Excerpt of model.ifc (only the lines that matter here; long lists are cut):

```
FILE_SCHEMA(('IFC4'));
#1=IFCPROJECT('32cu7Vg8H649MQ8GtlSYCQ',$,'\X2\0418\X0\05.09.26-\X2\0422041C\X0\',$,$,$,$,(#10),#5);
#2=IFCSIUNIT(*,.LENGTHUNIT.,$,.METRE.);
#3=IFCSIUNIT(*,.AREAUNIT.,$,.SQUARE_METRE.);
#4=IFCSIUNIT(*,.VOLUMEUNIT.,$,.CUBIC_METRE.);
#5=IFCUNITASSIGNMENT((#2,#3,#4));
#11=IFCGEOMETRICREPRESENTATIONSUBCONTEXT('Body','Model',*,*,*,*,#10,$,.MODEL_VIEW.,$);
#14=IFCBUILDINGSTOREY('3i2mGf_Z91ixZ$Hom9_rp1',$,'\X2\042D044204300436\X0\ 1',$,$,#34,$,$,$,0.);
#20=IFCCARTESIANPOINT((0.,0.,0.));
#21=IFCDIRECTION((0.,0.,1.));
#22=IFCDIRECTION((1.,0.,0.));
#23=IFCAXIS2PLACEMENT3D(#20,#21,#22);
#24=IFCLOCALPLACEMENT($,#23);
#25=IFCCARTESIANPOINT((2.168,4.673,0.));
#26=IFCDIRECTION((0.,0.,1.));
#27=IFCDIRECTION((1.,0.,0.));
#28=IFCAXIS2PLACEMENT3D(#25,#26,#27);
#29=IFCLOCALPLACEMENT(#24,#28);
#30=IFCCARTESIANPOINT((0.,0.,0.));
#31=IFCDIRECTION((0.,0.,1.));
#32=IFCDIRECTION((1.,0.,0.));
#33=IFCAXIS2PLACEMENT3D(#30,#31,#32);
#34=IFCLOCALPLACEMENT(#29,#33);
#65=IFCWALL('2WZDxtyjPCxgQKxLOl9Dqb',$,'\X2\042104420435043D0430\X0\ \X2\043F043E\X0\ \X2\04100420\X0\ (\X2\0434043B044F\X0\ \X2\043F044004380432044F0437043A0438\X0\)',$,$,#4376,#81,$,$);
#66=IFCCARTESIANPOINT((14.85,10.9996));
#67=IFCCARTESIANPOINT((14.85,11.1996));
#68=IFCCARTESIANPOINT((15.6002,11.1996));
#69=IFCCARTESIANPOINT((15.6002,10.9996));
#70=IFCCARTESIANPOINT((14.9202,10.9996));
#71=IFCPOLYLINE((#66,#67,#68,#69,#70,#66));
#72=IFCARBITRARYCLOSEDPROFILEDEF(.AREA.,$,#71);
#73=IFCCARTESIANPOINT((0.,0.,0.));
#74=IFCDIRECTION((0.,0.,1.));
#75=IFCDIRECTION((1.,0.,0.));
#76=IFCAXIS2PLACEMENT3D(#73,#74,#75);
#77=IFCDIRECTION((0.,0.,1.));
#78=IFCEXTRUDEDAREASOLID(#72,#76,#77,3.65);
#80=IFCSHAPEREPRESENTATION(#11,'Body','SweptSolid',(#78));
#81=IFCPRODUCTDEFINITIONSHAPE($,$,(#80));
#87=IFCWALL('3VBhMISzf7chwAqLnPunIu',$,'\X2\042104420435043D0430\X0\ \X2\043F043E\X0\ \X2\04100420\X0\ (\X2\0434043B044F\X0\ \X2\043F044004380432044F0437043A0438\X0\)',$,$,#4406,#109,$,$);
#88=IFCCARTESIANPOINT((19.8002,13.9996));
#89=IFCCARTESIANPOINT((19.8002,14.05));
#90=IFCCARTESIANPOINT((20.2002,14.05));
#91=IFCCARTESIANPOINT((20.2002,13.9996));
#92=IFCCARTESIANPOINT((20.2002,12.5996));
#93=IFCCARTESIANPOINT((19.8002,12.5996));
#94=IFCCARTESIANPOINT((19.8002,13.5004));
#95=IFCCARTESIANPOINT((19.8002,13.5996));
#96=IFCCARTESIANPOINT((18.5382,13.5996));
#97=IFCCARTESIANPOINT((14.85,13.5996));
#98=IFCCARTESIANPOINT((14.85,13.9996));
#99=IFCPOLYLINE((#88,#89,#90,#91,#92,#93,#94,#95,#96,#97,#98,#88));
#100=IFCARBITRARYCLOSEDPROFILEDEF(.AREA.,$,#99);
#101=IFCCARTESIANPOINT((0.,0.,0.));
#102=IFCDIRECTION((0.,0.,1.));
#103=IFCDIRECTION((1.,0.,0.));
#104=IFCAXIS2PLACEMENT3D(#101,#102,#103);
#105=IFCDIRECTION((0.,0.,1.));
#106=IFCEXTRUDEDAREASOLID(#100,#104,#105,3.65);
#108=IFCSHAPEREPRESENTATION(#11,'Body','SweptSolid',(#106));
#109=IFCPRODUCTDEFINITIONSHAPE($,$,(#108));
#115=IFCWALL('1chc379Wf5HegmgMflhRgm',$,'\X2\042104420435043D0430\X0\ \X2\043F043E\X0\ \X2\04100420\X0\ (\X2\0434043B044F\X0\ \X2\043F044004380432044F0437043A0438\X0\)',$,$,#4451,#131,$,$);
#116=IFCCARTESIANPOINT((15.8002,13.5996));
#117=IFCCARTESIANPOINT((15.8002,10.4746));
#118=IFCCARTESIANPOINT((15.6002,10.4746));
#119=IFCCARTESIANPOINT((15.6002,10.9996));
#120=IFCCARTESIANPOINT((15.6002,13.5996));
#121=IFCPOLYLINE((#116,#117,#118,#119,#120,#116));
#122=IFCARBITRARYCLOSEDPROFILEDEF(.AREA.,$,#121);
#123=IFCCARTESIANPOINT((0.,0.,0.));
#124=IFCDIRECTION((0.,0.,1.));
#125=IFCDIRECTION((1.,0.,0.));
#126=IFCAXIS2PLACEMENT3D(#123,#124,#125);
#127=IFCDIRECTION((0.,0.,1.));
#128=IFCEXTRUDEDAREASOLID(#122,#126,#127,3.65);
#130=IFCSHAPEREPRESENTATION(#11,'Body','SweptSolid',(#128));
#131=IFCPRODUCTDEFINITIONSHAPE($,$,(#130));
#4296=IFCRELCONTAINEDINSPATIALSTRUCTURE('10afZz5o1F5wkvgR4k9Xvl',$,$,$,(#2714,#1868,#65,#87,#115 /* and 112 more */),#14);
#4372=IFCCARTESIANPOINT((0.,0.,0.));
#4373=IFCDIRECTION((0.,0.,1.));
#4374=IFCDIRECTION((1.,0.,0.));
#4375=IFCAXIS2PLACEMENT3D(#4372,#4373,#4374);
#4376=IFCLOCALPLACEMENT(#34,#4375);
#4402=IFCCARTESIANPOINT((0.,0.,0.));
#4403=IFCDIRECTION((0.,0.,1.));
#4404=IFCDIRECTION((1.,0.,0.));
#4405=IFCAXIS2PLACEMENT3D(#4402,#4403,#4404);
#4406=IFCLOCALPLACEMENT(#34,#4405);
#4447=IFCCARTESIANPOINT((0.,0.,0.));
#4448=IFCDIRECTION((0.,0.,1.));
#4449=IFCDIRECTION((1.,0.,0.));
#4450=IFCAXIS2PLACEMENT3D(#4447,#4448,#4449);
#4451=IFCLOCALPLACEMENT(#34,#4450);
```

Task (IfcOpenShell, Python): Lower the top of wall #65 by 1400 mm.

```python
import ifcopenshell
import ifcopenshell.geom
import ifcopenshell.util.representation
import ifcopenshell.util.shape

model = ifcopenshell.open("model.ifc")
settings = ifcopenshell.geom.settings()


def volume(element):
    """Net volume in cubic metres, openings subtracted."""
    shape = ifcopenshell.geom.create_shape(settings, element)
    return ifcopenshell.util.shape.get_volume(shape.geometry)


wall = model.by_guid("2WZDxtyjPCxgQKxLOl9Dqb")
before = volume(wall)

body = ifcopenshell.util.representation.get_representation(wall, "Model", "Body")
solid = body.Items[0]
old_height = solid.Depth
solid.Depth -= 1.4
after = volume(wall)

print(f"height {old_height:g} -> {solid.Depth:g}, volume {before:.3f} -> {after:.3f} m3")

model.write("model-out.ifc")
```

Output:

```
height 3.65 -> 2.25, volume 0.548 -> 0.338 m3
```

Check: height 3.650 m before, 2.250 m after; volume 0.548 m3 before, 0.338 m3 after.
